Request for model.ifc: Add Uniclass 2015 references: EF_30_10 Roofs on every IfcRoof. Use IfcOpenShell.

First a look at what the model holds.

```python
import ifcopenshell

model = ifcopenshell.open("model.ifc")
print(model.schema)
print("classifications:", [c.Name for c in model.by_type("IfcClassification")])
for ifc_class in ("IfcDoor", "IfcRoof", "IfcStair", "IfcWall", "IfcWindow"):
    print(ifc_class, len(model.by_type(ifc_class)))
```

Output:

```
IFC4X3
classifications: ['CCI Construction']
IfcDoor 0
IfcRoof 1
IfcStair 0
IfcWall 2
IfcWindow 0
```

```python
import ifcopenshell
import ifcopenshell.api.classification

model = ifcopenshell.open("model.ifc")

system = ifcopenshell.api.classification.add_classification(model, classification="Uniclass 2015")

codes = {
    "IfcRoof": ("EF_30_10", "Roofs"),
}
for ifc_class, (code, name) in codes.items():
    products = model.by_type(ifc_class)
    ifcopenshell.api.classification.add_reference(
        model, products=products, classification=system, identification=code, name=name
    )
    print(code, len(products))

model.write("model_edited.ifc")
```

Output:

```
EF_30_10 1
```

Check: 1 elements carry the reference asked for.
